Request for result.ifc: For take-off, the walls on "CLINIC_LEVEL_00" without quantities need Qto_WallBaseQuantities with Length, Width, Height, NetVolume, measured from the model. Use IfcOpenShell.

First a look at what the model holds.

```python
import ifcopenshell
import ifcopenshell.util.element
import ifcopenshell.util.unit

model = ifcopenshell.open("result.ifc")
print(model.schema)
for unit_type in ("LENGTHUNIT", "AREAUNIT", "VOLUMEUNIT"):
    print(unit_type, ifcopenshell.util.unit.calculate_unit_scale(model, unit_type))
storey = next(s for s in model.by_type("IfcBuildingStorey") if s.Name == "CLINIC_LEVEL_00")
walls = [e for e in ifcopenshell.util.element.get_decomposition(storey) if e.is_a("IfcWall")]
for e in sorted(walls, key=lambda e: e.id()):
    print(e.id(), e.is_a(), e.Name, list(ifcopenshell.util.element.get_psets(e, qtos_only=True)), sep=" | ")
```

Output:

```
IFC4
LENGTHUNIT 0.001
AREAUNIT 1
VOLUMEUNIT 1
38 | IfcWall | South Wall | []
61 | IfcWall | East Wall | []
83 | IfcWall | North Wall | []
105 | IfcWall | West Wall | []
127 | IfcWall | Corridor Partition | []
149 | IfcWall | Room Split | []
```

```python
import ifcopenshell
import ifcopenshell.api.pset
import ifcopenshell.geom
import ifcopenshell.util.element
import ifcopenshell.util.shape
import ifcopenshell.util.unit

model = ifcopenshell.open("result.ifc")
unit_scale = ifcopenshell.util.unit.calculate_unit_scale(model)
volume_scale = ifcopenshell.util.unit.calculate_unit_scale(model, "VOLUMEUNIT")
settings = ifcopenshell.geom.settings()

storey = next(s for s in model.by_type("IfcBuildingStorey") if s.Name == "CLINIC_LEVEL_00")
walls = [e for e in ifcopenshell.util.element.get_decomposition(storey) if e.is_a("IfcWall")]

for e in sorted(walls, key=lambda e: e.id()):
    if ifcopenshell.util.element.get_psets(e, qtos_only=True, should_inherit=False):
        continue
    # Geometry comes back in metres, in the element's own axes.
    shape = ifcopenshell.geom.create_shape(settings, e)
    values = {
        "Length": ifcopenshell.util.shape.get_x(shape.geometry) / unit_scale,
        "Width": ifcopenshell.util.shape.get_y(shape.geometry) / unit_scale,
        "Height": ifcopenshell.util.shape.get_z(shape.geometry) / unit_scale,
        "NetVolume": ifcopenshell.util.shape.get_volume(shape.geometry) / volume_scale,
    }
    qto = ifcopenshell.api.pset.add_qto(model, product=e, name="Qto_WallBaseQuantities")
    ifcopenshell.api.pset.edit_qto(model, qto=qto, properties=values)
    print(e.id(), {k: round(v, 3) for k, v in values.items()})

model.write("result_edited.ifc")
```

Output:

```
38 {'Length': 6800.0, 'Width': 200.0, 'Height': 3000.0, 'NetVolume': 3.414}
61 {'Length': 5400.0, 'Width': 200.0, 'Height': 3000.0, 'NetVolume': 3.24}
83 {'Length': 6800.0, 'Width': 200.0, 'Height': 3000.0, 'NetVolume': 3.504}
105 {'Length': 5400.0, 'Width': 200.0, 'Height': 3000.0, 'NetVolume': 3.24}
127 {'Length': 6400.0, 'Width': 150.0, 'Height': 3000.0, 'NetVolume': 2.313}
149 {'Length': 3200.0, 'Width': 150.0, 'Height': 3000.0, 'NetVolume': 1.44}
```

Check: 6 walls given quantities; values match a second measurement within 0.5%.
